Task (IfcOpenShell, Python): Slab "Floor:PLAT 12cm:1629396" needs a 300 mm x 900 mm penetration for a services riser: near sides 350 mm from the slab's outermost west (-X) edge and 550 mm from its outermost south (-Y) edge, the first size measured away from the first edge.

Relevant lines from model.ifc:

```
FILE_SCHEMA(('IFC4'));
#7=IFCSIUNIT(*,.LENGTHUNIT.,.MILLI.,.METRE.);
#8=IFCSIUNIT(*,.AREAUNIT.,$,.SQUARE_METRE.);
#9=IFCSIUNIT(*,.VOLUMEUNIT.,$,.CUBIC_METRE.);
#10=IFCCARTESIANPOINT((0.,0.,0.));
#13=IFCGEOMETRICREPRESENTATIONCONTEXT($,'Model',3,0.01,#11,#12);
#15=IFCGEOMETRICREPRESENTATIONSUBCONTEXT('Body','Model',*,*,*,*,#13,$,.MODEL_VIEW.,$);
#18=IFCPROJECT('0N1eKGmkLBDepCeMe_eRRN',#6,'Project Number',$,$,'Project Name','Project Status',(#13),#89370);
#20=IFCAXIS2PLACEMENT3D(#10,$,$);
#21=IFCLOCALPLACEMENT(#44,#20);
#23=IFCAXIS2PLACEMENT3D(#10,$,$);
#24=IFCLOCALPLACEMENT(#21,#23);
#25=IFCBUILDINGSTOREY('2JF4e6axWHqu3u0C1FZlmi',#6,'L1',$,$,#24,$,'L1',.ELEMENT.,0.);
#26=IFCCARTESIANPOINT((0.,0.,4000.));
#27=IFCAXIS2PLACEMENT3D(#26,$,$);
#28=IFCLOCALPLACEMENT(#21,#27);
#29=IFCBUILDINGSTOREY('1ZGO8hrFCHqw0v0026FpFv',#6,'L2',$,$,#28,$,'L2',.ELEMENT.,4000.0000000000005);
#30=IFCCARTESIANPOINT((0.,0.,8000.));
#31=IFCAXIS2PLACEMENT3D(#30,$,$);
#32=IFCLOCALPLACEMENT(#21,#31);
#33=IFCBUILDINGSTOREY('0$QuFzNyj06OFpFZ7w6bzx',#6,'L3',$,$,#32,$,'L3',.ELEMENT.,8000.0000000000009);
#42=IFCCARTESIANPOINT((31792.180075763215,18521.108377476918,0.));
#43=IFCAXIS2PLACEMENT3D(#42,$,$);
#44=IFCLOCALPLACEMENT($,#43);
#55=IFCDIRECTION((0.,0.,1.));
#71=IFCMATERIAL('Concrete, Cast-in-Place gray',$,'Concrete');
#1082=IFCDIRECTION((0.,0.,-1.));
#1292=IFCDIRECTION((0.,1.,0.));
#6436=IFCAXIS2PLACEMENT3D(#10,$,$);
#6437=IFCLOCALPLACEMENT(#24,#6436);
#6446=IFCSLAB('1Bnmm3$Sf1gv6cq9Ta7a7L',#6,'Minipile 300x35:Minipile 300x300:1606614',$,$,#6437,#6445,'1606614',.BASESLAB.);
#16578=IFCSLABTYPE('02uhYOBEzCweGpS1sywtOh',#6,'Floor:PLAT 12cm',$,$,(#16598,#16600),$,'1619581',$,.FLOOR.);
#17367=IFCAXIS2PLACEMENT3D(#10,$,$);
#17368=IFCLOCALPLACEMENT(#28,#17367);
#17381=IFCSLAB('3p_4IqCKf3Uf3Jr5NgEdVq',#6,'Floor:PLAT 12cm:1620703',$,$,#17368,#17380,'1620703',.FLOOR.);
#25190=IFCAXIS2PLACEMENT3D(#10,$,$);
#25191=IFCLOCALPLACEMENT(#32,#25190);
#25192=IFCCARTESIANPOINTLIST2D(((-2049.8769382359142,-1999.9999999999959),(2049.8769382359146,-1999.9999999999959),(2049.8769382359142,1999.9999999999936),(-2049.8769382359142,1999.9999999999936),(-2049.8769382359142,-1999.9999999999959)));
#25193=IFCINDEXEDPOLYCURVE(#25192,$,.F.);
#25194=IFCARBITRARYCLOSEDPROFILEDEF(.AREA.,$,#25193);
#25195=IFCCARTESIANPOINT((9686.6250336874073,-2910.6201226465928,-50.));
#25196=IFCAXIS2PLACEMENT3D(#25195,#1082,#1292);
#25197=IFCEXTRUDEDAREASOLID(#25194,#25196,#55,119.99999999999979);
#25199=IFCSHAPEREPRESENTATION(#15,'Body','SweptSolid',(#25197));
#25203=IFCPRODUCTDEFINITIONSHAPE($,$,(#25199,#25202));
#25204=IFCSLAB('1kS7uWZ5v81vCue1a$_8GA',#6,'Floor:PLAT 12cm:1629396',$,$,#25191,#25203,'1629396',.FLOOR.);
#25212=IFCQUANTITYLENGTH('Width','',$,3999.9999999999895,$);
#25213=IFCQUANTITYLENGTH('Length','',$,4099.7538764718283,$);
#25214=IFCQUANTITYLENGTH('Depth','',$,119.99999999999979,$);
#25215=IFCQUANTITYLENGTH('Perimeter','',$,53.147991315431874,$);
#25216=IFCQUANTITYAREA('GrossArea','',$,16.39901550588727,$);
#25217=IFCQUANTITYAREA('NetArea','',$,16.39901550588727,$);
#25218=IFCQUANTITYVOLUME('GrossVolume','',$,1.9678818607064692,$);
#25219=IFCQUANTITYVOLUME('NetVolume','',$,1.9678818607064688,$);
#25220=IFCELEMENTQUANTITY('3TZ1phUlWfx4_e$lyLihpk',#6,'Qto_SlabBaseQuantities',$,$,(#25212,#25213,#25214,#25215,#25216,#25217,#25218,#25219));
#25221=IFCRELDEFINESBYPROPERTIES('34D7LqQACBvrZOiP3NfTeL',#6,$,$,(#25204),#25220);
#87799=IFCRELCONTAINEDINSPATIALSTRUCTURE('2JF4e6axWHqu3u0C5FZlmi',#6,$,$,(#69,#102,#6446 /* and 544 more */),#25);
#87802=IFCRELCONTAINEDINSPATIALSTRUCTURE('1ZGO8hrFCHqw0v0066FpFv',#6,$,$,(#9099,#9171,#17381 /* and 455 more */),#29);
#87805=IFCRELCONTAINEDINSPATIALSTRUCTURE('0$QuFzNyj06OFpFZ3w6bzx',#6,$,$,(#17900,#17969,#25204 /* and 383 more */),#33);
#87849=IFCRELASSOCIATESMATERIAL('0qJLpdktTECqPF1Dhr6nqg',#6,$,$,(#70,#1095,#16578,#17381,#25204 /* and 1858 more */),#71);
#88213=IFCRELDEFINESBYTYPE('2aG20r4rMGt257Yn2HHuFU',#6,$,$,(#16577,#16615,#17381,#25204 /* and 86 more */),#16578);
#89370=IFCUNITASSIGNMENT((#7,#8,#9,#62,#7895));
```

```python
import numpy as np
import ifcopenshell
import ifcopenshell.api.feature
import ifcopenshell.api.geometry
import ifcopenshell.api.pset
import ifcopenshell.api.root
import ifcopenshell.geom
import ifcopenshell.util.element
import ifcopenshell.util.placement
import ifcopenshell.util.representation
import ifcopenshell.util.shape
import ifcopenshell.util.unit

model = ifcopenshell.open("model.ifc")
unit_scale = ifcopenshell.util.unit.calculate_unit_scale(model)
area_scale = ifcopenshell.util.unit.calculate_unit_scale(model, "AREAUNIT")
volume_scale = ifcopenshell.util.unit.calculate_unit_scale(model, "VOLUMEUNIT")
settings = ifcopenshell.geom.settings()


def volume(element):
    """Net volume in cubic metres, openings subtracted."""
    shape = ifcopenshell.geom.create_shape(settings, element)
    return ifcopenshell.util.shape.get_volume(shape.geometry)


slab = model.by_guid("1kS7uWZ5v81vCue1a$_8GA")
before = volume(slab)

# Extent in the slab's own axes, in metres. The edges named are its -X and -Y sides.
slab_shape = ifcopenshell.geom.create_shape(settings, slab)
vertices = ifcopenshell.util.shape.get_vertices(slab_shape.geometry)
x_min, y_min, bottom = vertices.min(axis=0)
top = vertices[:, 2].max()

opening = ifcopenshell.api.root.create_entity(model, ifc_class="IfcOpeningElement", name="Services riser opening", predefined_type="OPENING")
context = ifcopenshell.util.representation.get_context(model, "Model", "Body", "MODEL_VIEW")
width, depth = 0.3, 0.9
outline = [(0.0, 0.0), (width, 0.0), (width, depth), (0.0, depth), (0.0, 0.0)]
# Overshoot both faces by 50 mm so the cut is clean.
shape = ifcopenshell.api.geometry.add_slab_representation(
    model, context=context, depth=top - bottom + 0.1, polyline=outline
)
ifcopenshell.api.geometry.assign_representation(model, product=opening, representation=shape)

matrix = ifcopenshell.util.placement.get_local_placement(slab.ObjectPlacement)
matrix[:, 3] = matrix @ np.append(np.array([x_min + 0.35, y_min + 0.55, bottom - 0.05]) / unit_scale, 1.0)
ifcopenshell.api.geometry.edit_object_placement(model, product=opening, matrix=matrix, is_si=False)
ifcopenshell.api.feature.add_feature(model, feature=opening, element=slab)

after = volume(slab)

# Update the slab's stored quantities.
qto = model.by_id(ifcopenshell.util.element.get_pset(slab, "Qto_SlabBaseQuantities", should_inherit=False)["id"])
ifcopenshell.api.pset.edit_qto(model, qto=qto, properties={
    "NetArea": after / (top - bottom) / area_scale,
    "NetVolume": after / volume_scale,
})

print(f"slab volume {before:.3f} -> {after:.3f} m3")

model.write("model-out.ifc")
```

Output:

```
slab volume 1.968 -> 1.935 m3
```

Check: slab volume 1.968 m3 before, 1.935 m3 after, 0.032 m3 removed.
